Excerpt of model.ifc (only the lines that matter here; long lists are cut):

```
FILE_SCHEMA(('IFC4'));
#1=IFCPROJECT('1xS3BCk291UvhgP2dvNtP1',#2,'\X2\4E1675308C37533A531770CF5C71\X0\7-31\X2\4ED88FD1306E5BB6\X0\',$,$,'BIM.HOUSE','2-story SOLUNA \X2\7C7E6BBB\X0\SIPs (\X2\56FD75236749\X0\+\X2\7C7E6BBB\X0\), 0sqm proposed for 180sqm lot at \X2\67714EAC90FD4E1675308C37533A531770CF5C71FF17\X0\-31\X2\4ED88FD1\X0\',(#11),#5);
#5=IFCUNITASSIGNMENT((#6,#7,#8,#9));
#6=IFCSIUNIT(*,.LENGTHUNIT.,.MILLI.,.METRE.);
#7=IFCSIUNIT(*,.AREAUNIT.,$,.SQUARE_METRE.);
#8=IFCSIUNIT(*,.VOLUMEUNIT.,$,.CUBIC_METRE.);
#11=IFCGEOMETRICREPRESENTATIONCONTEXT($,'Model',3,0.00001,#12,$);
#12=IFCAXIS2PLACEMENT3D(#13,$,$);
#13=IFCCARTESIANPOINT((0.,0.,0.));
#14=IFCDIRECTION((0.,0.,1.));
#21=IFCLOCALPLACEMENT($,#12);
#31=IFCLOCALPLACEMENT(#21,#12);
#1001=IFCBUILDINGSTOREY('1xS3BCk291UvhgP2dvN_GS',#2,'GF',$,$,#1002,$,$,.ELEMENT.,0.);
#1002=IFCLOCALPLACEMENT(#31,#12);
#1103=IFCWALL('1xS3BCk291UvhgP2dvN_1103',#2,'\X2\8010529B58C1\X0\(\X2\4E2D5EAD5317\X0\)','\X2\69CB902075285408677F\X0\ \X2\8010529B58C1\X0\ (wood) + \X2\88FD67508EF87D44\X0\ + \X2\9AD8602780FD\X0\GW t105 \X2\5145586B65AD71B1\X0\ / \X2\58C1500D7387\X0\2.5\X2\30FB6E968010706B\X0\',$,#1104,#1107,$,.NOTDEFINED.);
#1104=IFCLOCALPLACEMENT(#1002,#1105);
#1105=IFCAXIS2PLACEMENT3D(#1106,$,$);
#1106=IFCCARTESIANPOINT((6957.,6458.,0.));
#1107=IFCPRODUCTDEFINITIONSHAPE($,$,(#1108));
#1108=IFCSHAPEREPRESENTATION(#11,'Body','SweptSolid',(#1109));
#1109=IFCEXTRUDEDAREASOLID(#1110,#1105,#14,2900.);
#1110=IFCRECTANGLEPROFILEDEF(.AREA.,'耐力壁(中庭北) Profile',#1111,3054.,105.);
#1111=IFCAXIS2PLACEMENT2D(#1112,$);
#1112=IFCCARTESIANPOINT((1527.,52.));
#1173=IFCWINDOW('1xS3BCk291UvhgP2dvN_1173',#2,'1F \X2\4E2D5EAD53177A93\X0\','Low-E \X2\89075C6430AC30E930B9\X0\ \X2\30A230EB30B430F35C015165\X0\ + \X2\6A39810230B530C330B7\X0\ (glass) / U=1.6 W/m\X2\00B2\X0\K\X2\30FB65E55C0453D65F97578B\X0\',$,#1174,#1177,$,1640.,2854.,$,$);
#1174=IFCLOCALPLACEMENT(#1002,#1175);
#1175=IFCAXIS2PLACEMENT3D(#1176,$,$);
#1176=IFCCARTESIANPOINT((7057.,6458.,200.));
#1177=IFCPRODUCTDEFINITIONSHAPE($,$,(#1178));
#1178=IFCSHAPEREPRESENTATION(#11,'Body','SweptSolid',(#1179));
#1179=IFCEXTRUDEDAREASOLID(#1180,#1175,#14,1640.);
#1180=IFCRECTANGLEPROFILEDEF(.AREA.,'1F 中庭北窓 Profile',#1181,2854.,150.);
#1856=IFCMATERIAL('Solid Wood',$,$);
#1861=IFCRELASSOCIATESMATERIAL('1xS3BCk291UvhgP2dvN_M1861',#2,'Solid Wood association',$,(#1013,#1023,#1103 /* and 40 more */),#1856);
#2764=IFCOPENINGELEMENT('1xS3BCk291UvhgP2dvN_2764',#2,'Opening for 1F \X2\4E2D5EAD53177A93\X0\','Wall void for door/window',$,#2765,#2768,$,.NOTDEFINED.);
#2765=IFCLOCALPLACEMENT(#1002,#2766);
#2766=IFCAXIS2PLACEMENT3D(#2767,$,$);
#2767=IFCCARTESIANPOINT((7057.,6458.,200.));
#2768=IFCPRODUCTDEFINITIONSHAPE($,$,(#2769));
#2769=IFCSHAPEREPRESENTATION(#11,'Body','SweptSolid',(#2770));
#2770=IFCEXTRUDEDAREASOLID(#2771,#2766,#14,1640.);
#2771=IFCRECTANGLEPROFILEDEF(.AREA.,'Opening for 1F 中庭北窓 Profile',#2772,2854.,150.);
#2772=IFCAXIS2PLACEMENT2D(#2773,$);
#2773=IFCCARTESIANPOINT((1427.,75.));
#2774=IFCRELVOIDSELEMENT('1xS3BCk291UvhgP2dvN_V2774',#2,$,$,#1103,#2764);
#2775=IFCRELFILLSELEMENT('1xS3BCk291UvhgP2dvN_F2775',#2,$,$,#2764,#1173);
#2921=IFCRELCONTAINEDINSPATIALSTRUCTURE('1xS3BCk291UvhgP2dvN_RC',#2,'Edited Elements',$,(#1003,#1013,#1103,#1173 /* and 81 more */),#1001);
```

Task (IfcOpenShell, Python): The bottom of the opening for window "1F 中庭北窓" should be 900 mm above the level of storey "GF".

```python
import numpy as np
import ifcopenshell
import ifcopenshell.api.geometry
import ifcopenshell.geom
import ifcopenshell.util.element
import ifcopenshell.util.placement
import ifcopenshell.util.shape
import ifcopenshell.util.unit

model = ifcopenshell.open("model.ifc")
unit_scale = ifcopenshell.util.unit.calculate_unit_scale(model)

window = model.by_guid("1xS3BCk291UvhgP2dvN_1173")
opening = window.FillsVoids[0].RelatingOpeningElement
storey = ifcopenshell.util.element.get_container(window, ifc_class="IfcBuildingStorey")
level = ifcopenshell.util.placement.get_local_placement(storey.ObjectPlacement)[2, 3]

# The opening's origin need not be at the sill, so measure its lowest point.
shape = ifcopenshell.geom.create_shape(ifcopenshell.geom.settings(), opening)
bottom = ifcopenshell.util.shape.get_shape_bottom_elevation(shape, shape.geometry) / unit_scale
dz = level + 0.9 / unit_scale - bottom

shift = np.array([0.0, 0.0, dz])
# The window is not placed relative to its opening, so move both.
for product in (opening, window):
    matrix = ifcopenshell.util.placement.get_local_placement(product.ObjectPlacement)
    matrix[:3, 3] += shift
    ifcopenshell.api.geometry.edit_object_placement(model, product=product, matrix=matrix, is_si=False)

print(f"moved by {dz * unit_scale:+.3f} m")

model.write("model_updated.ifc")
```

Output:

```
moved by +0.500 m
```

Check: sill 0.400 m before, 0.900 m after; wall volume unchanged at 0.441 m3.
